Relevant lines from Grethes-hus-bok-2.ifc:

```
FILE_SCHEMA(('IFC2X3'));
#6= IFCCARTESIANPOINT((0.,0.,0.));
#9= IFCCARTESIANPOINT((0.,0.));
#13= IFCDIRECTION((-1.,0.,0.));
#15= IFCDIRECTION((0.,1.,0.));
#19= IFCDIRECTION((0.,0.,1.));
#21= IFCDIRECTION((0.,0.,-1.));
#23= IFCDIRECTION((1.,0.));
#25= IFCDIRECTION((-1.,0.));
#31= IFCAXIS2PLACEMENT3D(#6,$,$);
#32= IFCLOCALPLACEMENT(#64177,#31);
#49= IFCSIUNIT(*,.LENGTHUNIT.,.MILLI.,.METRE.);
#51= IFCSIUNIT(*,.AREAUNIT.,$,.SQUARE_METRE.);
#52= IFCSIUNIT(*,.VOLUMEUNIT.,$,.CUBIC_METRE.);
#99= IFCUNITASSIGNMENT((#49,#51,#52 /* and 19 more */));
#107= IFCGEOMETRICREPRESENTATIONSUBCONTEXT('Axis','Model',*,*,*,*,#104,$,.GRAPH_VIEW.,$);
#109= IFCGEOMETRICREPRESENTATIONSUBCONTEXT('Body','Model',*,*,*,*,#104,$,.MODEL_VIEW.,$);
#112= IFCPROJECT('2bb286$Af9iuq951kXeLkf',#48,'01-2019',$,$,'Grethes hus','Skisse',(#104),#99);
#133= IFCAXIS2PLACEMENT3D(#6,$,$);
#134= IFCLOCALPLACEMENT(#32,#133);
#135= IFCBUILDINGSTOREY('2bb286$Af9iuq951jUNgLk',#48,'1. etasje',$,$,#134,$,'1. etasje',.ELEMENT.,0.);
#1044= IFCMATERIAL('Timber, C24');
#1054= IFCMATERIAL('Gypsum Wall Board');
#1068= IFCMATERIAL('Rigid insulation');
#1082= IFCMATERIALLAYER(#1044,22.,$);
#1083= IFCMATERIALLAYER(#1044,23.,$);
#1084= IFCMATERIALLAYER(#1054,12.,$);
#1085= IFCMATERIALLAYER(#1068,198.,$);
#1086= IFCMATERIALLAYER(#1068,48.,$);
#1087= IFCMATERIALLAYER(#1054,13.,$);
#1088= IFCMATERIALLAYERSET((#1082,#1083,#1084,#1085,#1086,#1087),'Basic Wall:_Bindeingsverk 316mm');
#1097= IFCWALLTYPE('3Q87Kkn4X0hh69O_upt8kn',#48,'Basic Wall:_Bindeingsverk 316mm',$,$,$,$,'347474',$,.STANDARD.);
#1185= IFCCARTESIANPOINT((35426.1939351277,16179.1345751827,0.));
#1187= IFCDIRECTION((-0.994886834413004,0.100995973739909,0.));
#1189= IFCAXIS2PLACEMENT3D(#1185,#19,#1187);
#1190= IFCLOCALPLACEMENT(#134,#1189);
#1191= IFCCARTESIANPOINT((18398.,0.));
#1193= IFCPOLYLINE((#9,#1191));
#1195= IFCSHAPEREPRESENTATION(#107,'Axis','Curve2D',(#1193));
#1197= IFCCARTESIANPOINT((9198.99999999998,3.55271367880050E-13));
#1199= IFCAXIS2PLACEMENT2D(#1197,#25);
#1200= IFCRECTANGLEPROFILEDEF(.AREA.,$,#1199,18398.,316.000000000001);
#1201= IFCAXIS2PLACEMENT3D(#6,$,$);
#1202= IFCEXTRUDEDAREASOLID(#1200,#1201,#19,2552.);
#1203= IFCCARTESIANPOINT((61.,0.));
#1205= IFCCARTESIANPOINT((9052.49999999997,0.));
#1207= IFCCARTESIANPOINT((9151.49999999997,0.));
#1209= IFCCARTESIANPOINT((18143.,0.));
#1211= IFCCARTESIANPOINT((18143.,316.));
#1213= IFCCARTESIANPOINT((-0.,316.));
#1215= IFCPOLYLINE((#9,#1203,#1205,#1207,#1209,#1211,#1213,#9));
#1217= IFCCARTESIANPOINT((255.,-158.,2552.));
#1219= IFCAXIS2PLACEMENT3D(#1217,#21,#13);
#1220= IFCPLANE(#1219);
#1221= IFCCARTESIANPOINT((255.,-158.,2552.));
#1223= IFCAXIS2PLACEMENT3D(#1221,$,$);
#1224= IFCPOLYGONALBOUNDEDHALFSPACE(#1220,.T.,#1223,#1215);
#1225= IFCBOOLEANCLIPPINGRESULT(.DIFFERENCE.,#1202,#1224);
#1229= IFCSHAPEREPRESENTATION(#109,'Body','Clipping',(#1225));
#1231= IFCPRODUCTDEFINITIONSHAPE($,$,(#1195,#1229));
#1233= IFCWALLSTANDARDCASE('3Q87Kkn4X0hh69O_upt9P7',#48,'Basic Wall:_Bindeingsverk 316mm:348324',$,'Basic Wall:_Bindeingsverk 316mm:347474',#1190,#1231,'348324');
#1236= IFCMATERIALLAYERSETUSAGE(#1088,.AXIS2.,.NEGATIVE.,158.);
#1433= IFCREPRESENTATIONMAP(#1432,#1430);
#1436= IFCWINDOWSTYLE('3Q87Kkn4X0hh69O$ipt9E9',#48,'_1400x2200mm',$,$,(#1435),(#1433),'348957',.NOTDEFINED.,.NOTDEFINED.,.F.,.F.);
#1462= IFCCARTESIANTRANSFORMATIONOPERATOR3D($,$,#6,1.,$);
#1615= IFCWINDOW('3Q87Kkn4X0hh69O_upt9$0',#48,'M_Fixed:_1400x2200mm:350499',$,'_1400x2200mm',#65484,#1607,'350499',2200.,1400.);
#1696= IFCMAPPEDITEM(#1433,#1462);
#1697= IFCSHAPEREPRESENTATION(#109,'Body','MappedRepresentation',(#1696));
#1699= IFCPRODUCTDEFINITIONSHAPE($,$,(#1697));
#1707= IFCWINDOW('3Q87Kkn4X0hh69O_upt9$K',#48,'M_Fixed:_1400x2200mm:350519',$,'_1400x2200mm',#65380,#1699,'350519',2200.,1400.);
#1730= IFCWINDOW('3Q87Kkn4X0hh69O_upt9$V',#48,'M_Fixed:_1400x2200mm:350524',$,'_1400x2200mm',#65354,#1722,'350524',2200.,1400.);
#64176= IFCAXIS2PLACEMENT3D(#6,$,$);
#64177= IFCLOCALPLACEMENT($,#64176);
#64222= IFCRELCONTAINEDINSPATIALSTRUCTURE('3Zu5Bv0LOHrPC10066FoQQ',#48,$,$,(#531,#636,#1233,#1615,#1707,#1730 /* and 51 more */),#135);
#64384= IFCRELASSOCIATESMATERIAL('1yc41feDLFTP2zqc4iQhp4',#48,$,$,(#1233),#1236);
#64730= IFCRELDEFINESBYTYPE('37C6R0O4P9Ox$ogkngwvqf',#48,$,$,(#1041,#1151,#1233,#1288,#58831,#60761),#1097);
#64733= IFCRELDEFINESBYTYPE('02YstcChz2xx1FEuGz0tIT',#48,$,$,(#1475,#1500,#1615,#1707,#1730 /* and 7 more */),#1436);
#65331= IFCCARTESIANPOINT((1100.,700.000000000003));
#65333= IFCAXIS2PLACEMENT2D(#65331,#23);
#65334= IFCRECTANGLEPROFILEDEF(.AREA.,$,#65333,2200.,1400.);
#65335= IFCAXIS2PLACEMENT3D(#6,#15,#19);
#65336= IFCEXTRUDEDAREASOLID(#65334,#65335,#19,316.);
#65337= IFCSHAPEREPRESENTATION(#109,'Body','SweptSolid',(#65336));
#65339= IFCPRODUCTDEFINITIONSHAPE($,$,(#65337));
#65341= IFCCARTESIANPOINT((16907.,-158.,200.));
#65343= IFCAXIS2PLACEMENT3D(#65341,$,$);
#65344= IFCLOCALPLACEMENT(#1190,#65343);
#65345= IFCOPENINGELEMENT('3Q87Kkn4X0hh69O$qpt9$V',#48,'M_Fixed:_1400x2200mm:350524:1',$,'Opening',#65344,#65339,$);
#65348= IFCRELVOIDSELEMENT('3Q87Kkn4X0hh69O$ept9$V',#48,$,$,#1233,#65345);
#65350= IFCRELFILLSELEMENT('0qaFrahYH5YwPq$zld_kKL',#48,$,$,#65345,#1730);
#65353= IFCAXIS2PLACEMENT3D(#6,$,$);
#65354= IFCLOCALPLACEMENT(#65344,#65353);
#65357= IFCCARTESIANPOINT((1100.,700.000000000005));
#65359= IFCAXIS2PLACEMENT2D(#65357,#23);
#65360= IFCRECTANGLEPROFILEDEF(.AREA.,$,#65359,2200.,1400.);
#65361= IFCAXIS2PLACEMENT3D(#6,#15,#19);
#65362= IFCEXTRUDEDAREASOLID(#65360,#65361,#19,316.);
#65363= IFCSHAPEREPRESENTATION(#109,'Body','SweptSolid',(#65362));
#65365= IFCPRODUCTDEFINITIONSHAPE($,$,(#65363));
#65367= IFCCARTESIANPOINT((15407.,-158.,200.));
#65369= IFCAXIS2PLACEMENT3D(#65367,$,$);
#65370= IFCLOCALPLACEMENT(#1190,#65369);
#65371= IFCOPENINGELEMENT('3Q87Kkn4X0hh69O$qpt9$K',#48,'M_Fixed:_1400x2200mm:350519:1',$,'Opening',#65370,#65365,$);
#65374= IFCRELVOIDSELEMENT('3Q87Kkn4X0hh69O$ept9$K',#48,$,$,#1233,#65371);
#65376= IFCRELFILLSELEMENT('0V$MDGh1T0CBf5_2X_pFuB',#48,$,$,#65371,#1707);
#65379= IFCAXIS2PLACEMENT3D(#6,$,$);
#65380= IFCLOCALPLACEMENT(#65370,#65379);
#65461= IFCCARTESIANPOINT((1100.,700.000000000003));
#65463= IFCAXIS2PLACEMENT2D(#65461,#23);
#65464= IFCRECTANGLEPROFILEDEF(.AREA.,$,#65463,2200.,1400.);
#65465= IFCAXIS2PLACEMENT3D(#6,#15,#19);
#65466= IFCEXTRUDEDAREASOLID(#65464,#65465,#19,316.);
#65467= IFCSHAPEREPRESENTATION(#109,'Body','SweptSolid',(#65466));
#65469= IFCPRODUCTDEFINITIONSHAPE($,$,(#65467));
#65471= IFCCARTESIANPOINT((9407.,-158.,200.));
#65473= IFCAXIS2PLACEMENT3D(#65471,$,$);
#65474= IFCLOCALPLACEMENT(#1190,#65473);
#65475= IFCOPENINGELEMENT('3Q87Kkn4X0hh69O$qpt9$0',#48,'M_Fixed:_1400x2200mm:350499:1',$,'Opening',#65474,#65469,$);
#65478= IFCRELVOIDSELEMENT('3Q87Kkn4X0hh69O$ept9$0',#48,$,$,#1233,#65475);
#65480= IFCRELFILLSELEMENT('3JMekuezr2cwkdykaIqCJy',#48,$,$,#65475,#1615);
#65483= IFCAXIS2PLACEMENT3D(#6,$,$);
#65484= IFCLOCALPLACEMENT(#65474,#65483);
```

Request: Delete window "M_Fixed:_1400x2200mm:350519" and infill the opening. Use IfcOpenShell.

```python
import ifcopenshell
import ifcopenshell.api.feature
import ifcopenshell.api.root
import ifcopenshell.geom
import ifcopenshell.util.shape

model = ifcopenshell.open("Grethes-hus-bok-2.ifc")
settings = ifcopenshell.geom.settings()


def volume(element):
    """Net volume in cubic metres, openings subtracted."""
    shape = ifcopenshell.geom.create_shape(settings, element)
    return ifcopenshell.util.shape.get_volume(shape.geometry)


window = model.by_guid("3Q87Kkn4X0hh69O_upt9$K")
opening = window.FillsVoids[0].RelatingOpeningElement
wall = opening.VoidsElements[0].RelatingBuildingElement
before = volume(wall)

ifcopenshell.api.root.remove_product(model, product=window)
ifcopenshell.api.feature.remove_feature(model, feature=opening)

after = volume(wall)

print(f"wall volume {before:.3f} -> {after:.3f} m3")

model.write("Grethes-hus-bok-2_v2.ifc")
```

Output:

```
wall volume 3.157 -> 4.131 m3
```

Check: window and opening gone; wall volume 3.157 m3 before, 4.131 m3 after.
